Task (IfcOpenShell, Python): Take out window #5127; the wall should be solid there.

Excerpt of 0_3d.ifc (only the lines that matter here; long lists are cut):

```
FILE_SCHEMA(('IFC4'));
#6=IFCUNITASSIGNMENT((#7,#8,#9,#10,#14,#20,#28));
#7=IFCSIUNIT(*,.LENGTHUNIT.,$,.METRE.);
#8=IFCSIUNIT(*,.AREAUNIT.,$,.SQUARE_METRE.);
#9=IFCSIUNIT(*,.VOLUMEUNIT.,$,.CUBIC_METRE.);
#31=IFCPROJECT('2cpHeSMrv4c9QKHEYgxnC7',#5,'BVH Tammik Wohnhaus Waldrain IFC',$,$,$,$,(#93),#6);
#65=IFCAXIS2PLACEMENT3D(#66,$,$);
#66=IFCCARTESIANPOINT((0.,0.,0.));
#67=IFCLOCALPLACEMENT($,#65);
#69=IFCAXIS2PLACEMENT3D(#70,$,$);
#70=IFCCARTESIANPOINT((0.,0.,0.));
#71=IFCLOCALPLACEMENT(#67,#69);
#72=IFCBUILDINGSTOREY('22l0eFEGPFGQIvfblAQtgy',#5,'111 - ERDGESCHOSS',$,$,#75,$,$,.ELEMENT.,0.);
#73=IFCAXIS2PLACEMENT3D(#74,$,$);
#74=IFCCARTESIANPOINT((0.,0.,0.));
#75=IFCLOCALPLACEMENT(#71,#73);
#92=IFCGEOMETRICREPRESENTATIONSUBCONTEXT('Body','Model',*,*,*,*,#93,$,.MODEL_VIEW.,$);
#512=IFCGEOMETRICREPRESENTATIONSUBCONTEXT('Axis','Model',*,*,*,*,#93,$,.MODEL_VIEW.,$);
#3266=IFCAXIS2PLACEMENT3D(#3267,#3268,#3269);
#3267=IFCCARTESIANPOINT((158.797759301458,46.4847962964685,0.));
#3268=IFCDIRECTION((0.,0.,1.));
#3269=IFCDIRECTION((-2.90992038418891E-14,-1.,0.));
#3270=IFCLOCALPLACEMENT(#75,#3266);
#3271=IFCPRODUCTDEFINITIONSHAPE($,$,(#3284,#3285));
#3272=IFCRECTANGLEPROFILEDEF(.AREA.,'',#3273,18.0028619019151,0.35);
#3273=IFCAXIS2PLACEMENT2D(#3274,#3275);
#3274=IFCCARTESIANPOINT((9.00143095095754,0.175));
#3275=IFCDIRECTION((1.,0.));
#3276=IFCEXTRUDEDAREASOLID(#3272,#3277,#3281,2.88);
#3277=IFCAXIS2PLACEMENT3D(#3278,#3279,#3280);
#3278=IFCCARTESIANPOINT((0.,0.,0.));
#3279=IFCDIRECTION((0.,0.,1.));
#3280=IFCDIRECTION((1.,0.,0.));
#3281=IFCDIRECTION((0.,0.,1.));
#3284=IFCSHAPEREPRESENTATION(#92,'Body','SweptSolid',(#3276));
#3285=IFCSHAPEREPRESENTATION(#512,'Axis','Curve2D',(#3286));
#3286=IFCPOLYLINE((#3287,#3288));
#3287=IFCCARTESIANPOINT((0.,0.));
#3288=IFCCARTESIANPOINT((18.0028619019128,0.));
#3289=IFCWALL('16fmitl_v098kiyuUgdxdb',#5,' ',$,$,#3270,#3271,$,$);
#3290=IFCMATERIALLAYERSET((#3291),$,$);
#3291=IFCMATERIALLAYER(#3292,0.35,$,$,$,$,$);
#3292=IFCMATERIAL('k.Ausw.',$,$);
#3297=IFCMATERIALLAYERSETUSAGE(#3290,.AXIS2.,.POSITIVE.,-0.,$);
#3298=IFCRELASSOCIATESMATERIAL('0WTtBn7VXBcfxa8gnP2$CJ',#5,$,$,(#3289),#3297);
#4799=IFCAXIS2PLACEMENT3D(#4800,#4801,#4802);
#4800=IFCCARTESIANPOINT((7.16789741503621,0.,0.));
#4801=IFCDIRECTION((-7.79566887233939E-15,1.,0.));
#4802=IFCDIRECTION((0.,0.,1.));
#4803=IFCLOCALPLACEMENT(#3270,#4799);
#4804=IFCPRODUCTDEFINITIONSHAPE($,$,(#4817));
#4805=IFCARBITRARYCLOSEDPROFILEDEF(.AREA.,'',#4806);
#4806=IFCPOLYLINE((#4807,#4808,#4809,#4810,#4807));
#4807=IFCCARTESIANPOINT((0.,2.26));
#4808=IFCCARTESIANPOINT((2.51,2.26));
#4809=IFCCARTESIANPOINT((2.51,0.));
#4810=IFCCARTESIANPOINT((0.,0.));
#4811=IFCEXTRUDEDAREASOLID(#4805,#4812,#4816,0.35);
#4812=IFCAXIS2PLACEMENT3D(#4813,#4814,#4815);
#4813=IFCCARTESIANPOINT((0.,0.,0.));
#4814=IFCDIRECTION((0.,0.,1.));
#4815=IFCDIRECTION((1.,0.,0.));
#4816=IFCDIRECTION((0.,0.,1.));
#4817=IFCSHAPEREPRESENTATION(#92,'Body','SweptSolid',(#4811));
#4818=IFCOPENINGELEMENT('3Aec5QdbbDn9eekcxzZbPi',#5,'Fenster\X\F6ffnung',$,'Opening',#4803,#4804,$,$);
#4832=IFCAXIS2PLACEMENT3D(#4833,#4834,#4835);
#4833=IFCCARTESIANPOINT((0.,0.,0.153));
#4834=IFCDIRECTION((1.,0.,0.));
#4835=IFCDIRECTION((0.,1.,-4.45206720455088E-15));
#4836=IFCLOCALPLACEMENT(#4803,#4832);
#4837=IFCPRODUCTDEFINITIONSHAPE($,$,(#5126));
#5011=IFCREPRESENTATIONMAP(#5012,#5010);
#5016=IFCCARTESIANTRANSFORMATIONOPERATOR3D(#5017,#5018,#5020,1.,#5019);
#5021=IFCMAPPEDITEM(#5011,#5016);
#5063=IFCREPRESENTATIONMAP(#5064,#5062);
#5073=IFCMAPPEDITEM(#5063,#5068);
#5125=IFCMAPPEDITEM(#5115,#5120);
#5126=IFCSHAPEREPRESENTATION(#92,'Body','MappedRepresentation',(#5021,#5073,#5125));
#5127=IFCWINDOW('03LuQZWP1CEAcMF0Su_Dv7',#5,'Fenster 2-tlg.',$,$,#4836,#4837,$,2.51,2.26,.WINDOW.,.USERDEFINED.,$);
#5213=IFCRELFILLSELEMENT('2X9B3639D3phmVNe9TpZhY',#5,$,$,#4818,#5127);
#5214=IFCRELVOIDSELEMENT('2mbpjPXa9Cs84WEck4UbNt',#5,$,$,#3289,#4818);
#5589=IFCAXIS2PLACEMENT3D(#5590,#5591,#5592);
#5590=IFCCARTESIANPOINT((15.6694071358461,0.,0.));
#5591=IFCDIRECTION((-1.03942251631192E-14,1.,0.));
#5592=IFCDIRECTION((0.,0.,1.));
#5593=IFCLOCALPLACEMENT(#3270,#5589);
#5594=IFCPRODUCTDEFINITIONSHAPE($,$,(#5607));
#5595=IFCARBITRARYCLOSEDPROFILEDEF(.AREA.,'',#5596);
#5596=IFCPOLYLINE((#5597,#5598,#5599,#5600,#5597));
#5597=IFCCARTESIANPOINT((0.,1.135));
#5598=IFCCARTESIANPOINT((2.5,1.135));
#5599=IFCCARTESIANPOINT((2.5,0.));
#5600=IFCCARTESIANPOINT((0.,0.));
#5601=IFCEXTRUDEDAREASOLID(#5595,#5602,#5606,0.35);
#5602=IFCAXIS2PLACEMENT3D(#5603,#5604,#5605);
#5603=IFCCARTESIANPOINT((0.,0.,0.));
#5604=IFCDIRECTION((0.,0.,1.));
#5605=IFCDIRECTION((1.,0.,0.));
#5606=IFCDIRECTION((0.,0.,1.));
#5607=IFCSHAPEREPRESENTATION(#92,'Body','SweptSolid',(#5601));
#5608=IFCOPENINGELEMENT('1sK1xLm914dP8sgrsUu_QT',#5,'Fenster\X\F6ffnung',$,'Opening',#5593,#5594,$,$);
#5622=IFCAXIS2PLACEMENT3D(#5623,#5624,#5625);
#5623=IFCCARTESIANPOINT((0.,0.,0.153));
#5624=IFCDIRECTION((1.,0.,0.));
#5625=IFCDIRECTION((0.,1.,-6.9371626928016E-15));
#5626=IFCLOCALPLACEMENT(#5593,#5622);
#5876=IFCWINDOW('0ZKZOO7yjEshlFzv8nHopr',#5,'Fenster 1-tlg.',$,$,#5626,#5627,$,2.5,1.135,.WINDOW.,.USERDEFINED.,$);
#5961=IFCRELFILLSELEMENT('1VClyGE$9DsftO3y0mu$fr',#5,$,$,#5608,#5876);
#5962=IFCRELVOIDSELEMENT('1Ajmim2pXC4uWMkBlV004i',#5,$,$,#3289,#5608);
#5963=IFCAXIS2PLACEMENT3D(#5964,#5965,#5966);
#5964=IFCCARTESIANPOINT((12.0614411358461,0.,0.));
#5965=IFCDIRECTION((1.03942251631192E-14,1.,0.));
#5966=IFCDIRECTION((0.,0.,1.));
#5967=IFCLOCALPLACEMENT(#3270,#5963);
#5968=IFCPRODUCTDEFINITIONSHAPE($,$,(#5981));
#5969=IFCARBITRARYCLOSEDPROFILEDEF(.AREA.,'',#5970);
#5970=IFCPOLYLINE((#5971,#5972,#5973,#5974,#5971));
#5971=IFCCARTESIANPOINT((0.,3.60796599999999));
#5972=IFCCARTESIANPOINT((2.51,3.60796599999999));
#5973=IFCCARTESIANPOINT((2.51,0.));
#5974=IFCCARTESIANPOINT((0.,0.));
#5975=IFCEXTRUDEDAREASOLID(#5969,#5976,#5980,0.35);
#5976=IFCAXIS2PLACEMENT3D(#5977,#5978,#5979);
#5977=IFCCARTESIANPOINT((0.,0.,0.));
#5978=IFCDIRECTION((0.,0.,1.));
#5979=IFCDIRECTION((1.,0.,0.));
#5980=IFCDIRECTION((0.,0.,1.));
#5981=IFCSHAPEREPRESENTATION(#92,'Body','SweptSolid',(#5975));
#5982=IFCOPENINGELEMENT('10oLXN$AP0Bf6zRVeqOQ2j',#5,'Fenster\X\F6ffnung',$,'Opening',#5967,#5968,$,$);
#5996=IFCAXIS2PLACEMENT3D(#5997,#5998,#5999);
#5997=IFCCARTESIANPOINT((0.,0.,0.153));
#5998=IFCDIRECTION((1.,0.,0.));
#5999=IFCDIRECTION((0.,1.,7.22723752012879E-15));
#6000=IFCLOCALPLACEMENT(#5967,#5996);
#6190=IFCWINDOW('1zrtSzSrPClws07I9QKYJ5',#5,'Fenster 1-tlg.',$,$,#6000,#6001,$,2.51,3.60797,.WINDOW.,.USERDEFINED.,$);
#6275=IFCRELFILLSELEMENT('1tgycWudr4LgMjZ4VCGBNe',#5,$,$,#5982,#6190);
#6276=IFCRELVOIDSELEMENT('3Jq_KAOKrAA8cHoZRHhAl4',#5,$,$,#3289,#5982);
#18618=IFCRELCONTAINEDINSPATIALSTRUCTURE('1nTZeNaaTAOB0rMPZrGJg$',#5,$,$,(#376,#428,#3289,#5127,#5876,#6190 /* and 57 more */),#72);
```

```python
import ifcopenshell
import ifcopenshell.api.feature
import ifcopenshell.api.root
import ifcopenshell.geom
import ifcopenshell.util.shape

model = ifcopenshell.open("0_3d.ifc")
settings = ifcopenshell.geom.settings()


def volume(element):
    """Net volume in cubic metres, openings subtracted."""
    shape = ifcopenshell.geom.create_shape(settings, element)
    return ifcopenshell.util.shape.get_volume(shape.geometry)


window = model.by_guid("03LuQZWP1CEAcMF0Su_Dv7")
opening = window.FillsVoids[0].RelatingOpeningElement
wall = opening.VoidsElements[0].RelatingBuildingElement
before = volume(wall)

ifcopenshell.api.root.remove_product(model, product=window)
ifcopenshell.api.feature.remove_feature(model, feature=opening)

after = volume(wall)

print(f"wall volume {before:.3f} -> {after:.3f} m3")

model.write("0_3d-out.ifc")
```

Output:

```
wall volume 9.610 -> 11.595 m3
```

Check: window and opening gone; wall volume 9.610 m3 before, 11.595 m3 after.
